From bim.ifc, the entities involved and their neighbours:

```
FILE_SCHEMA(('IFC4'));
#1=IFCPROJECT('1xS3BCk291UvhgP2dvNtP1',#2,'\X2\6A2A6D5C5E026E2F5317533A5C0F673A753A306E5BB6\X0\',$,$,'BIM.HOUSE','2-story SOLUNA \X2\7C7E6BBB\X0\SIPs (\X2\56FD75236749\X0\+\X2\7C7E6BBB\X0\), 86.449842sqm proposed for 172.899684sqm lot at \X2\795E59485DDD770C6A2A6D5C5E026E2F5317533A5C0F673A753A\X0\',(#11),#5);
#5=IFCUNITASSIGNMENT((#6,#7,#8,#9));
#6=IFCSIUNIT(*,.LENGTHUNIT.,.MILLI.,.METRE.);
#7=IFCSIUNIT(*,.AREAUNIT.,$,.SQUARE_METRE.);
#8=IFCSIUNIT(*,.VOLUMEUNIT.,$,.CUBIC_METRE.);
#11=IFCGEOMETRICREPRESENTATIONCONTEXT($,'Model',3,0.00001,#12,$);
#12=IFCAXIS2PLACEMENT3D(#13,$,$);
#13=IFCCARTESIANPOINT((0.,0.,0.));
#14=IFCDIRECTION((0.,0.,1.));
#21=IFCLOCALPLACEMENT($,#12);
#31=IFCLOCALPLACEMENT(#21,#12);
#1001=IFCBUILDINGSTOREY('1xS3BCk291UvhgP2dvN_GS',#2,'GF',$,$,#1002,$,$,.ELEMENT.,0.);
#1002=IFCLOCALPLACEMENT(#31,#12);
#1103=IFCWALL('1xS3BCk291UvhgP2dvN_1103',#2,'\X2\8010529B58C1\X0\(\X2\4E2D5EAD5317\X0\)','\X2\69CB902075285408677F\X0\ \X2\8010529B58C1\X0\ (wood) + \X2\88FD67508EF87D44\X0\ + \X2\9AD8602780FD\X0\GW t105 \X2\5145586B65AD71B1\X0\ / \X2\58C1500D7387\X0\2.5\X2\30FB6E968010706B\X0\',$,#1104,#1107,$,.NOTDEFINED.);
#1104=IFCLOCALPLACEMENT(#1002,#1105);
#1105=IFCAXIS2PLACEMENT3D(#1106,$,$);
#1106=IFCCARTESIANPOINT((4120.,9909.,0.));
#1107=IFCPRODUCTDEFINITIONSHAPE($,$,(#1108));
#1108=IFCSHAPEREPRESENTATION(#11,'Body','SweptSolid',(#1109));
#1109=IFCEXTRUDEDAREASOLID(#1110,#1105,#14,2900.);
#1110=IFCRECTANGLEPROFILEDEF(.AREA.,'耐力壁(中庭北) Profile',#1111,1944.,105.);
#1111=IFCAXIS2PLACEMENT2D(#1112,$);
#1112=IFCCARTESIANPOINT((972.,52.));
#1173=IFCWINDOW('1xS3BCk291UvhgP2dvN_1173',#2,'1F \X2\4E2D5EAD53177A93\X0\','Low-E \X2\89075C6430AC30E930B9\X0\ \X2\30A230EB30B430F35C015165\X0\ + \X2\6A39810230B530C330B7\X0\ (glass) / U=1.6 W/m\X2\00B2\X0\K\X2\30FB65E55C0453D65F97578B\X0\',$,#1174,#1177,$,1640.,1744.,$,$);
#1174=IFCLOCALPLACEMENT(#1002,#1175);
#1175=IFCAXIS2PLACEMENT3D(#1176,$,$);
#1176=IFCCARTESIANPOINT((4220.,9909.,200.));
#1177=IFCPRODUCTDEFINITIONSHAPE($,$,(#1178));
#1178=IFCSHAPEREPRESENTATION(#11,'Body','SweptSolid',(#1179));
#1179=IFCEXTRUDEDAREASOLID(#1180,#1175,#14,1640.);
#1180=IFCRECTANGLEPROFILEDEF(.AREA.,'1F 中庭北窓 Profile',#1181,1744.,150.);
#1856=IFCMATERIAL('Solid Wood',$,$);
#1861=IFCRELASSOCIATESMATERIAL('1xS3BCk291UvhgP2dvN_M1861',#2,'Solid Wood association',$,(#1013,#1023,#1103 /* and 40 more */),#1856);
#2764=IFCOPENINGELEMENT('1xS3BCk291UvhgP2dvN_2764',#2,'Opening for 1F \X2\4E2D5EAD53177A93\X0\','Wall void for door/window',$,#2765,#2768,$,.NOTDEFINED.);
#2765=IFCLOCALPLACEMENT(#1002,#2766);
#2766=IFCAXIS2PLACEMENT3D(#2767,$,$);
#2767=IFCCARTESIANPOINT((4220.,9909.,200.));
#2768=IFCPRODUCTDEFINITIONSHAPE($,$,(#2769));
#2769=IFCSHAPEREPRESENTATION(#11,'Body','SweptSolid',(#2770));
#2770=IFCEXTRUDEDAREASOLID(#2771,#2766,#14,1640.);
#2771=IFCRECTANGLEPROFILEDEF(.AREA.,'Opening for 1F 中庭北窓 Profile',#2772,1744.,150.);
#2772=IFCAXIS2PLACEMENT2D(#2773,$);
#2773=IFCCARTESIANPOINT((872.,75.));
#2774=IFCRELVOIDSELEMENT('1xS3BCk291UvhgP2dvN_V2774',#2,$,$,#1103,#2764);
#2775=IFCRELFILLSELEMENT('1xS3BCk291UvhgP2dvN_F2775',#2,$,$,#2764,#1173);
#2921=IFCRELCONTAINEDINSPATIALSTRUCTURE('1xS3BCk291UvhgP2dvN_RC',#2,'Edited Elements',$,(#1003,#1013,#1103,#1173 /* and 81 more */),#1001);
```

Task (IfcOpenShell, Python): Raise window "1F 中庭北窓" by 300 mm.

```python
import numpy as np
import ifcopenshell
import ifcopenshell.api.geometry
import ifcopenshell.util.placement
import ifcopenshell.util.unit

model = ifcopenshell.open("bim.ifc")
unit_scale = ifcopenshell.util.unit.calculate_unit_scale(model)

window = model.by_id(1173)
opening = window.FillsVoids[0].RelatingOpeningElement
dz = 300.0

shift = np.array([0.0, 0.0, dz])
# The window is not placed relative to its opening, so move both.
for product in (opening, window):
    matrix = ifcopenshell.util.placement.get_local_placement(product.ObjectPlacement)
    matrix[:3, 3] += shift
    ifcopenshell.api.geometry.edit_object_placement(model, product=product, matrix=matrix, is_si=False)

print(f"moved by {dz * unit_scale:+.3f} m")

model.write("bim-out.ifc")
```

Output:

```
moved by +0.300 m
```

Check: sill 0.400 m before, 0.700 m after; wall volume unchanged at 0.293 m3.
